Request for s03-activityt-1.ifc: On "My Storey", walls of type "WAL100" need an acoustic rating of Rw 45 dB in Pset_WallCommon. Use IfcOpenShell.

First a look at what the model holds.

```python
import ifcopenshell
import ifcopenshell.util.element

model = ifcopenshell.open("s03-activityt-1.ifc")
print(model.schema)
storey = next(s for s in model.by_type("IfcBuildingStorey") if s.Name == "My Storey")
walls = [e for e in ifcopenshell.util.element.get_decomposition(storey) if e.is_a("IfcWall")]
seen = {}
for e in walls:
    element_type = ifcopenshell.util.element.get_type(e)
    key = (element_type.Name if element_type != e and element_type else None, ifcopenshell.util.element.get_pset(e, "Pset_WallCommon", "AcousticRating"))
    seen[key] = seen.get(key, 0) + 1
for (name, value), count in sorted(seen.items(), key=str):
    print(count, "x", name, "|", value)
```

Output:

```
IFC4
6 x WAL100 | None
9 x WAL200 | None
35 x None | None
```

```python
import ifcopenshell
import ifcopenshell.api.pset
import ifcopenshell.util.element

model = ifcopenshell.open("s03-activityt-1.ifc")

storey = next(s for s in model.by_type("IfcBuildingStorey") if s.Name == "My Storey")
walls = [e for e in ifcopenshell.util.element.get_decomposition(storey) if e.is_a("IfcWall")]

count = 0
for e in walls:
    element_type = ifcopenshell.util.element.get_type(e)
    if element_type in (None, e) or element_type.Name != "WAL100":
        continue
    # add_pset returns the element's existing set when there is one.
    pset = ifcopenshell.api.pset.add_pset(model, product=e, name="Pset_WallCommon")
    ifcopenshell.api.pset.edit_pset(model, pset=pset, properties={"AcousticRating": "Rw 45 dB"})
    count += 1

print(count, "walls updated")

model.write("s03-activityt-1-out.ifc")
```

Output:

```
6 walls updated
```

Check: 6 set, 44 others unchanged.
